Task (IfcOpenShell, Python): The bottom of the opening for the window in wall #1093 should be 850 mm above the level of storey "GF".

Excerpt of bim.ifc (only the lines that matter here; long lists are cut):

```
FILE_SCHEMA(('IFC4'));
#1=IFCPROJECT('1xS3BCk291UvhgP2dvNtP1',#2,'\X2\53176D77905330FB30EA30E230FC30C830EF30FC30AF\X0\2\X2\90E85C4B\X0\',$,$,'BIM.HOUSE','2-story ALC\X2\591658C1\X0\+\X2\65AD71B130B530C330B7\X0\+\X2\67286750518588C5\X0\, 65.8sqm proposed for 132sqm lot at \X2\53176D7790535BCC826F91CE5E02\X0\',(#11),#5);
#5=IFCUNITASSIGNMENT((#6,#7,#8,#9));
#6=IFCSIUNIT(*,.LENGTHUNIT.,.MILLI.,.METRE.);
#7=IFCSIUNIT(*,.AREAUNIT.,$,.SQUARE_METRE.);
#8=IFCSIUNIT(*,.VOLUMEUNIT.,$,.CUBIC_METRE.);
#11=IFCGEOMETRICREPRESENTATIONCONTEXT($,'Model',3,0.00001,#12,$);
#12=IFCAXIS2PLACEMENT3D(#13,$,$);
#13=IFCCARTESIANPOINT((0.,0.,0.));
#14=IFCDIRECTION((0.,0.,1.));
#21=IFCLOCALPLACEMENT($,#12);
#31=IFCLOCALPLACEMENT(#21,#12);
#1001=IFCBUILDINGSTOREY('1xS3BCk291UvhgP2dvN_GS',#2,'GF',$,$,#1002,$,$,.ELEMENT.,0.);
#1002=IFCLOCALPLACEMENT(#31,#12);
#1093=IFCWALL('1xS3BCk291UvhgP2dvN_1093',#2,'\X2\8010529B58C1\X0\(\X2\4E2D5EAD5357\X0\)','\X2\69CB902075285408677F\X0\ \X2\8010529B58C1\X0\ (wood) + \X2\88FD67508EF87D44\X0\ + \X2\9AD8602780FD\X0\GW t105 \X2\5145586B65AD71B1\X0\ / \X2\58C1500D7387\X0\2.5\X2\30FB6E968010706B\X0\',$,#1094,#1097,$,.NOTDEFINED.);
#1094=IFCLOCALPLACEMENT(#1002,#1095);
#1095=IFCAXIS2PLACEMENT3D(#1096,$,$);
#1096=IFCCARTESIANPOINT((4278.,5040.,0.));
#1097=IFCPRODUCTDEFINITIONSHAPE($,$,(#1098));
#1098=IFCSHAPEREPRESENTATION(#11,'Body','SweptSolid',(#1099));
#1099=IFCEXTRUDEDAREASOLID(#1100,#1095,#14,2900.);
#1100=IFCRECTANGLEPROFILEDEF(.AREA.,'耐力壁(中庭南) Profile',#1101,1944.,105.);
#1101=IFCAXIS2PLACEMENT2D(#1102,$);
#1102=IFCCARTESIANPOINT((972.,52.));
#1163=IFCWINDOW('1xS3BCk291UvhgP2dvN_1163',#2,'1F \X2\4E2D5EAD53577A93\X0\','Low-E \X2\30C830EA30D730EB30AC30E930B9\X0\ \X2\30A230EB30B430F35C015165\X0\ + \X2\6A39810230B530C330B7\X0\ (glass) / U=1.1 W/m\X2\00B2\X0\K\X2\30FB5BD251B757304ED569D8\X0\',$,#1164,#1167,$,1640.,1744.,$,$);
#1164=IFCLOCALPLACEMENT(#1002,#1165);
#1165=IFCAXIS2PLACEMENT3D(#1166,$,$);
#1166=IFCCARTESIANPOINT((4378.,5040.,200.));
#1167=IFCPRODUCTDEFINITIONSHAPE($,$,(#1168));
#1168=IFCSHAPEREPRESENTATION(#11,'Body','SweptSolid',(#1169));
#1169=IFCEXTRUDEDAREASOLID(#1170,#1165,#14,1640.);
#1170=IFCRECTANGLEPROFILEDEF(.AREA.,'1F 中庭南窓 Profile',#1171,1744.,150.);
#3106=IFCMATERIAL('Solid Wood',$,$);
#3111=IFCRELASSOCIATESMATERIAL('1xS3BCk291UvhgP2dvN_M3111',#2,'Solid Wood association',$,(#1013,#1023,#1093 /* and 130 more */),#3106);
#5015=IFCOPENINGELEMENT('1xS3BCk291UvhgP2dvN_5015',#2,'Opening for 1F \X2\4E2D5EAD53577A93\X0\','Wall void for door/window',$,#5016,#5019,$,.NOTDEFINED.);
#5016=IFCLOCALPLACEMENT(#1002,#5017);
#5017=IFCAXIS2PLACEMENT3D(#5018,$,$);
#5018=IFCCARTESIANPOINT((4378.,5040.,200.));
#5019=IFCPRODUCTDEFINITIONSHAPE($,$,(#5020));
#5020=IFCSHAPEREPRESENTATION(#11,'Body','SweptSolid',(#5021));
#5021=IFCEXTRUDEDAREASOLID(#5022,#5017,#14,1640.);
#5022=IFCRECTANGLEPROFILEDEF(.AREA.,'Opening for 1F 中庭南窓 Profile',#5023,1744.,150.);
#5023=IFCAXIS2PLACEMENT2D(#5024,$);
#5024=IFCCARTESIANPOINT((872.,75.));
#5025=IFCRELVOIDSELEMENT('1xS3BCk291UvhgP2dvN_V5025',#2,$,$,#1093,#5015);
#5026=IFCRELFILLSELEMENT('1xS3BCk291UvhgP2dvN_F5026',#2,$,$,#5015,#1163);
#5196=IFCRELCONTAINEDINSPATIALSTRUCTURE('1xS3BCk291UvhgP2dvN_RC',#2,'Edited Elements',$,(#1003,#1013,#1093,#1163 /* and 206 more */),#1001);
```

```python
import numpy as np
import ifcopenshell
import ifcopenshell.api.geometry
import ifcopenshell.geom
import ifcopenshell.util.element
import ifcopenshell.util.placement
import ifcopenshell.util.shape
import ifcopenshell.util.unit

model = ifcopenshell.open("bim.ifc")
unit_scale = ifcopenshell.util.unit.calculate_unit_scale(model)

window = model.by_id(1163)
opening = window.FillsVoids[0].RelatingOpeningElement
storey = ifcopenshell.util.element.get_container(window, ifc_class="IfcBuildingStorey")
level = ifcopenshell.util.placement.get_local_placement(storey.ObjectPlacement)[2, 3]

# The opening's origin need not be at the sill, so measure its lowest point.
shape = ifcopenshell.geom.create_shape(ifcopenshell.geom.settings(), opening)
bottom = ifcopenshell.util.shape.get_shape_bottom_elevation(shape, shape.geometry) / unit_scale
dz = level + 0.85 / unit_scale - bottom

shift = np.array([0.0, 0.0, dz])
# The window is not placed relative to its opening, so move both.
for product in (opening, window):
    matrix = ifcopenshell.util.placement.get_local_placement(product.ObjectPlacement)
    matrix[:3, 3] += shift
    ifcopenshell.api.geometry.edit_object_placement(model, product=product, matrix=matrix, is_si=False)

print(f"moved by {dz * unit_scale:+.3f} m")

model.write("bim_v2.ifc")
```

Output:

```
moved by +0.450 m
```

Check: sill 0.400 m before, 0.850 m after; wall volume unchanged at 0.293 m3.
